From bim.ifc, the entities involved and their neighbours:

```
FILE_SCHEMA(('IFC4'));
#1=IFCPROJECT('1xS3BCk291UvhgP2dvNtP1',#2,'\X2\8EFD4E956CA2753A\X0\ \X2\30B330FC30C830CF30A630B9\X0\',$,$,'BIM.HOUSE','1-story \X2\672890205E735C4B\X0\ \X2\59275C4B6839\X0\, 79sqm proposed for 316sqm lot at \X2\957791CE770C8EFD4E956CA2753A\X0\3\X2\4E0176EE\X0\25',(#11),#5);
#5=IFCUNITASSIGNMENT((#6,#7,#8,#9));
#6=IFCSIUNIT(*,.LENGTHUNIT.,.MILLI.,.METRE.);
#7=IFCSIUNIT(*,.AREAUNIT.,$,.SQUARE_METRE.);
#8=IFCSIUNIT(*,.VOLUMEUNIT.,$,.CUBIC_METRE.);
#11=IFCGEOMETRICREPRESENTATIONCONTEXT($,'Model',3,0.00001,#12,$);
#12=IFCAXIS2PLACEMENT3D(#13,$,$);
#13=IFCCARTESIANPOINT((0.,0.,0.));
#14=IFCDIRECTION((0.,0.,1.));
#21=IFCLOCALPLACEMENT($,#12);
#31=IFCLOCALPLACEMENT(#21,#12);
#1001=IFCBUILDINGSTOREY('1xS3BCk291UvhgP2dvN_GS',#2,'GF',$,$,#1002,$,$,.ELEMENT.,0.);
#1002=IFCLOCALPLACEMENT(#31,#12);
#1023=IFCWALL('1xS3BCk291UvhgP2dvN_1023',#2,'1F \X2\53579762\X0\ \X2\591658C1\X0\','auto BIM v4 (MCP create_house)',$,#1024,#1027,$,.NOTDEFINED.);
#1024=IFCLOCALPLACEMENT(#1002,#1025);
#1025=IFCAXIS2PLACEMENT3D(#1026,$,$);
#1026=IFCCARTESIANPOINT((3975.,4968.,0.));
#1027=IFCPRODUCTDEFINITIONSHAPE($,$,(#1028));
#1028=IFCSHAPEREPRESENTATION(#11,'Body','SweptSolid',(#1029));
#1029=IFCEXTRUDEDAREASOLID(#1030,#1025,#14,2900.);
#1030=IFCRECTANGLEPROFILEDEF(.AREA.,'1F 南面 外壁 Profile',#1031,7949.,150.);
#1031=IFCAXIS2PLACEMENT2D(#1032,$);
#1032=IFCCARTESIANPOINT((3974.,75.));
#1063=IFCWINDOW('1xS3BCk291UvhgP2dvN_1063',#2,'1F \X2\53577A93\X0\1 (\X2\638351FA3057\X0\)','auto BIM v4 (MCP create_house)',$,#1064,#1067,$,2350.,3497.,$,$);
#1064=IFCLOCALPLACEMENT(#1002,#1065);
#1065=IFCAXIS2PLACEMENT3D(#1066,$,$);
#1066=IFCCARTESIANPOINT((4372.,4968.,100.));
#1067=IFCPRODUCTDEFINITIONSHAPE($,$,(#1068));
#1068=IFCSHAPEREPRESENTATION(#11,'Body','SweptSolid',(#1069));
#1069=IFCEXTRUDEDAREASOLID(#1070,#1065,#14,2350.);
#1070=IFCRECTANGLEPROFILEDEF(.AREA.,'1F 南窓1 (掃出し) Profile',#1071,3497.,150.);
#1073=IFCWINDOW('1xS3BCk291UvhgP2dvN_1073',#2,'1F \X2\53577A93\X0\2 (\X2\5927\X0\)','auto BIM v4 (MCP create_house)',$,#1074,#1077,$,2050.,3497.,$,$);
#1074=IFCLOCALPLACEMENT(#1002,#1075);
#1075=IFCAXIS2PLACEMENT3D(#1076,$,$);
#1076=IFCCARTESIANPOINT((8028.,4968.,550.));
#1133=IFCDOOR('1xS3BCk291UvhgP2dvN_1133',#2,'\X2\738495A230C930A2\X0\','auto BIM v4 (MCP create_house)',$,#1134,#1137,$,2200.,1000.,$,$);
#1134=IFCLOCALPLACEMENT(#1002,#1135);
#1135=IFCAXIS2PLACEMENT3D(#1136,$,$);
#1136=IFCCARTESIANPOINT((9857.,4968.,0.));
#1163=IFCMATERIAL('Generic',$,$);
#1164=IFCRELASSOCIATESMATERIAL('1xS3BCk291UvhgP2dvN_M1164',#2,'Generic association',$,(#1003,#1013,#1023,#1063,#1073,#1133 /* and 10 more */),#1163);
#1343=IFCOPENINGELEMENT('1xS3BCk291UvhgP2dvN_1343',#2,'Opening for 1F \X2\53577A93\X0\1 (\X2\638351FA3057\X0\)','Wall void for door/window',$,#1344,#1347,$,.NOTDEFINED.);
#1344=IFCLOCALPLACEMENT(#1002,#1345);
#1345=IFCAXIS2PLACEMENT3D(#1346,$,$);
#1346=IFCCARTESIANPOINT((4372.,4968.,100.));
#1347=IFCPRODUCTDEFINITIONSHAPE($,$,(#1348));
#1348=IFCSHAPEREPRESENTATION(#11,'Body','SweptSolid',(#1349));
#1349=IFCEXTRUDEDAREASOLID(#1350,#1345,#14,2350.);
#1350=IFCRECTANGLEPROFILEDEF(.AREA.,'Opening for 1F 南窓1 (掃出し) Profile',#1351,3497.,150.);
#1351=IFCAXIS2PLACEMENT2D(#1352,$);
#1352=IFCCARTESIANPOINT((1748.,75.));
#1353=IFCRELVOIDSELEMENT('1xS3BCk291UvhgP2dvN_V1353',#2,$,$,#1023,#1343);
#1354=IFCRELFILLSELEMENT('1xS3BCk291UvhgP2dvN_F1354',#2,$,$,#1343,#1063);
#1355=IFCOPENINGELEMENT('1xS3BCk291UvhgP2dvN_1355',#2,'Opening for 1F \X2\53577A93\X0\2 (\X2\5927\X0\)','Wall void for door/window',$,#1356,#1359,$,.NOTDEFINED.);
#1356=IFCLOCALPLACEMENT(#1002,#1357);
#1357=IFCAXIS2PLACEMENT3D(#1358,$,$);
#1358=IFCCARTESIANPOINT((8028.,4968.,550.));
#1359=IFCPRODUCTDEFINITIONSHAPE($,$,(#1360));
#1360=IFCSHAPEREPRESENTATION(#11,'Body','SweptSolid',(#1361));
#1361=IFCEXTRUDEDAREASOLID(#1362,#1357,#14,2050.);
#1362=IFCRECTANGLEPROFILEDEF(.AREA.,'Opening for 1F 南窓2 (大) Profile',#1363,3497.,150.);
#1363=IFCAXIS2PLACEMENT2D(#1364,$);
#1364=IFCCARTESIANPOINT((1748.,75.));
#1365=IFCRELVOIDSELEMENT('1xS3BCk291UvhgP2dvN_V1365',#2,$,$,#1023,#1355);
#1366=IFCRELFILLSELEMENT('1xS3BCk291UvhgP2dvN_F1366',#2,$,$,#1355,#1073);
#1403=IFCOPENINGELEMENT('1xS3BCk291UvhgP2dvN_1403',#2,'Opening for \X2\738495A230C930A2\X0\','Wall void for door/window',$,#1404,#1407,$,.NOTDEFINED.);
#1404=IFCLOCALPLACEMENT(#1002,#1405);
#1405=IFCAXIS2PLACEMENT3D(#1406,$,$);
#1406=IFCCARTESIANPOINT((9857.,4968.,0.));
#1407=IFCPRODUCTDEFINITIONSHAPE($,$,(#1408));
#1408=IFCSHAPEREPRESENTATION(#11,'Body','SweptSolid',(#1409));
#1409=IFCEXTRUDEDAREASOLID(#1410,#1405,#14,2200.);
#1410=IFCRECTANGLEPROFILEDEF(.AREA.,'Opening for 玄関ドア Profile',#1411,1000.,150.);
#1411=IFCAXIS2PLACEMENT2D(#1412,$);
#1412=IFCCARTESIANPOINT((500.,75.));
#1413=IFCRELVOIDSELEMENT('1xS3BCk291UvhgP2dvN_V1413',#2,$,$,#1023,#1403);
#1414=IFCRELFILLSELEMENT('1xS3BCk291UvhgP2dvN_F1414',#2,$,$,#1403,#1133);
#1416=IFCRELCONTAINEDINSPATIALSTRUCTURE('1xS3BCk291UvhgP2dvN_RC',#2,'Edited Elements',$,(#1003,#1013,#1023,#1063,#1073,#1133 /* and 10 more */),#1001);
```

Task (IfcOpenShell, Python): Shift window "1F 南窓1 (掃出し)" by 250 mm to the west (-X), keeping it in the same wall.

```python
import ifcopenshell
import ifcopenshell.api.geometry
import ifcopenshell.util.placement
import ifcopenshell.util.unit

model = ifcopenshell.open("bim.ifc")
unit_scale = ifcopenshell.util.unit.calculate_unit_scale(model)

window = model.by_guid("1xS3BCk291UvhgP2dvN_1063")
opening = window.FillsVoids[0].RelatingOpeningElement
wall = opening.VoidsElements[0].RelatingBuildingElement

wall_matrix = ifcopenshell.util.placement.get_local_placement(wall.ObjectPlacement)
shift = wall_matrix[:3, 0] * -0.25 / unit_scale
before = ifcopenshell.util.placement.get_local_placement(window.ObjectPlacement)[:3, 3].copy()

# The window is not placed relative to its opening, so move both.
for product in (opening, window):
    matrix = ifcopenshell.util.placement.get_local_placement(product.ObjectPlacement)
    matrix[:3, 3] += shift
    ifcopenshell.api.geometry.edit_object_placement(model, product=product, matrix=matrix, is_si=False)

after = ifcopenshell.util.placement.get_local_placement(window.ObjectPlacement)[:3, 3]
print("window moved by", (after - before).round(3) + 0.0)

model.write("bim_rev.ifc")
```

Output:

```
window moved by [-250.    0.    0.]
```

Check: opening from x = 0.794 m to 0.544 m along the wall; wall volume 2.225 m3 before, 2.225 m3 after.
